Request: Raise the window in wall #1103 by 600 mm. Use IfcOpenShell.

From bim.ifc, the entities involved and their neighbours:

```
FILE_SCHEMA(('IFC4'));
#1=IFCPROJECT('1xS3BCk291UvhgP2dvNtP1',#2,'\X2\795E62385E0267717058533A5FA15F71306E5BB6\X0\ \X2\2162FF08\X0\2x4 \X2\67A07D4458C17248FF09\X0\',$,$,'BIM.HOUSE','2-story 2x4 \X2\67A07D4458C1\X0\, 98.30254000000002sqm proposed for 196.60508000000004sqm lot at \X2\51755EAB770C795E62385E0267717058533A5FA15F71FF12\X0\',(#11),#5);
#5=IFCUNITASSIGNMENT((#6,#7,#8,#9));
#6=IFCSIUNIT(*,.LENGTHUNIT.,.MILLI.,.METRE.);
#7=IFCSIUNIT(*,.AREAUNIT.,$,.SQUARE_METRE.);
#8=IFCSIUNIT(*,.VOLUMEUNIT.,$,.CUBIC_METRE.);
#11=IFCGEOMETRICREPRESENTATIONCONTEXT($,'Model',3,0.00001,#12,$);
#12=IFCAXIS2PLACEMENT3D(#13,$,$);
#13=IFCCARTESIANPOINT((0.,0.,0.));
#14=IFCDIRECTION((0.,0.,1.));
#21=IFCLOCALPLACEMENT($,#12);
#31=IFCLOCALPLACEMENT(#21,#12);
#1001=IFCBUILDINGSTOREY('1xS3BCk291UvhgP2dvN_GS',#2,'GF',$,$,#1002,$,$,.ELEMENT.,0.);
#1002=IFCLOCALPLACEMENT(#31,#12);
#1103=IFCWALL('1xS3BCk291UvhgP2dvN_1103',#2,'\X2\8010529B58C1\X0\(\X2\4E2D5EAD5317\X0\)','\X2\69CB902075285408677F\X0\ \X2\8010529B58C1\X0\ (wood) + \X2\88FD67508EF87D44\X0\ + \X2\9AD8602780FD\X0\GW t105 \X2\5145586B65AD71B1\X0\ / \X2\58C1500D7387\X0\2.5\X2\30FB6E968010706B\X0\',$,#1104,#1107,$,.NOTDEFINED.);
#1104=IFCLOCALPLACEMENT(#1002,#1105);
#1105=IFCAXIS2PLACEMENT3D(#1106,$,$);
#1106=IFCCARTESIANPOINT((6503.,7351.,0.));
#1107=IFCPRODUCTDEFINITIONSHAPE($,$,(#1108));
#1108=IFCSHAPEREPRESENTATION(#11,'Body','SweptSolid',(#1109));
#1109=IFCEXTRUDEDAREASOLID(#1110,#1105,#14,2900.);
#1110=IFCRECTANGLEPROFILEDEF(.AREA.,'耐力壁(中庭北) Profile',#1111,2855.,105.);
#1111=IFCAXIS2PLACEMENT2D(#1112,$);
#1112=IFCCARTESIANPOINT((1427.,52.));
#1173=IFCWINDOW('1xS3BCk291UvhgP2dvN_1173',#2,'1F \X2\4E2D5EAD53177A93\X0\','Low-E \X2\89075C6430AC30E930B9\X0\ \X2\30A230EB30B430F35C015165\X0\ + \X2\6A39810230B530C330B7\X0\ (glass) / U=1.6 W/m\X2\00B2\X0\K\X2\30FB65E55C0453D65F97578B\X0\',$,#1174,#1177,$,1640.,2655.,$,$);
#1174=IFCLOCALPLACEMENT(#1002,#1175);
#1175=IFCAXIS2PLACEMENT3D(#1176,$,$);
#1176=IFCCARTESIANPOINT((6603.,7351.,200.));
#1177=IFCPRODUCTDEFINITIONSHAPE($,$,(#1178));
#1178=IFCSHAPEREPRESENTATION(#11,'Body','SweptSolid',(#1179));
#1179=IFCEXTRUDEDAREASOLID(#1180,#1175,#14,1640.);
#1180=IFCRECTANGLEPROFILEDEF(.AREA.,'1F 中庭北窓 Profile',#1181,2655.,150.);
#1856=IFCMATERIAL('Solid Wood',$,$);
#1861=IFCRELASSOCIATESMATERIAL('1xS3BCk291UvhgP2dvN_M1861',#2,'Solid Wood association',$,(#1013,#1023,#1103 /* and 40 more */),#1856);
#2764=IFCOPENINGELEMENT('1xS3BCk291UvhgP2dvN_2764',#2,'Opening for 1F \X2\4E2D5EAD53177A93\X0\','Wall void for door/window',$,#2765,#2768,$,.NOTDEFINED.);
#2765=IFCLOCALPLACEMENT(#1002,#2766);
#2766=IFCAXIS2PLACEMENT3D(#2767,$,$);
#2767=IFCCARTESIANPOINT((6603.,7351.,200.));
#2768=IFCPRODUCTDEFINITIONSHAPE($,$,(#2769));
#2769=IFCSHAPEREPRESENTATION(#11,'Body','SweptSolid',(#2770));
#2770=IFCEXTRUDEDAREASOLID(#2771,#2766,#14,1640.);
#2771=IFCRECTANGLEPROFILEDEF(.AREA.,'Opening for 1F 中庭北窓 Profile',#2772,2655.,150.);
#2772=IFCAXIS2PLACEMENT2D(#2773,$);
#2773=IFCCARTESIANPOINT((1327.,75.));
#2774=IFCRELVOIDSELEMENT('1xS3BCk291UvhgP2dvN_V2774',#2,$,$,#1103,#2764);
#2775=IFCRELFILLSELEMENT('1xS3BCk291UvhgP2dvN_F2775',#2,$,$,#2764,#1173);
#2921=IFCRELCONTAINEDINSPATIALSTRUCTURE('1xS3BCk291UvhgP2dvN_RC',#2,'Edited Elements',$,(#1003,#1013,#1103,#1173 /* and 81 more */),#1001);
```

```python
import numpy as np
import ifcopenshell
import ifcopenshell.api.geometry
import ifcopenshell.util.placement
import ifcopenshell.util.unit

model = ifcopenshell.open("bim.ifc")
unit_scale = ifcopenshell.util.unit.calculate_unit_scale(model)

window = model.by_id(1173)
opening = window.FillsVoids[0].RelatingOpeningElement
dz = 600.0

shift = np.array([0.0, 0.0, dz])
# The window is not placed relative to its opening, so move both.
for product in (opening, window):
    matrix = ifcopenshell.util.placement.get_local_placement(product.ObjectPlacement)
    matrix[:3, 3] += shift
    ifcopenshell.api.geometry.edit_object_placement(model, product=product, matrix=matrix, is_si=False)

print(f"moved by {dz * unit_scale:+.3f} m")

model.write("bim-out.ifc")
```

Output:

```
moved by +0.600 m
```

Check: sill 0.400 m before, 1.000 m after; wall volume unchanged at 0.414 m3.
